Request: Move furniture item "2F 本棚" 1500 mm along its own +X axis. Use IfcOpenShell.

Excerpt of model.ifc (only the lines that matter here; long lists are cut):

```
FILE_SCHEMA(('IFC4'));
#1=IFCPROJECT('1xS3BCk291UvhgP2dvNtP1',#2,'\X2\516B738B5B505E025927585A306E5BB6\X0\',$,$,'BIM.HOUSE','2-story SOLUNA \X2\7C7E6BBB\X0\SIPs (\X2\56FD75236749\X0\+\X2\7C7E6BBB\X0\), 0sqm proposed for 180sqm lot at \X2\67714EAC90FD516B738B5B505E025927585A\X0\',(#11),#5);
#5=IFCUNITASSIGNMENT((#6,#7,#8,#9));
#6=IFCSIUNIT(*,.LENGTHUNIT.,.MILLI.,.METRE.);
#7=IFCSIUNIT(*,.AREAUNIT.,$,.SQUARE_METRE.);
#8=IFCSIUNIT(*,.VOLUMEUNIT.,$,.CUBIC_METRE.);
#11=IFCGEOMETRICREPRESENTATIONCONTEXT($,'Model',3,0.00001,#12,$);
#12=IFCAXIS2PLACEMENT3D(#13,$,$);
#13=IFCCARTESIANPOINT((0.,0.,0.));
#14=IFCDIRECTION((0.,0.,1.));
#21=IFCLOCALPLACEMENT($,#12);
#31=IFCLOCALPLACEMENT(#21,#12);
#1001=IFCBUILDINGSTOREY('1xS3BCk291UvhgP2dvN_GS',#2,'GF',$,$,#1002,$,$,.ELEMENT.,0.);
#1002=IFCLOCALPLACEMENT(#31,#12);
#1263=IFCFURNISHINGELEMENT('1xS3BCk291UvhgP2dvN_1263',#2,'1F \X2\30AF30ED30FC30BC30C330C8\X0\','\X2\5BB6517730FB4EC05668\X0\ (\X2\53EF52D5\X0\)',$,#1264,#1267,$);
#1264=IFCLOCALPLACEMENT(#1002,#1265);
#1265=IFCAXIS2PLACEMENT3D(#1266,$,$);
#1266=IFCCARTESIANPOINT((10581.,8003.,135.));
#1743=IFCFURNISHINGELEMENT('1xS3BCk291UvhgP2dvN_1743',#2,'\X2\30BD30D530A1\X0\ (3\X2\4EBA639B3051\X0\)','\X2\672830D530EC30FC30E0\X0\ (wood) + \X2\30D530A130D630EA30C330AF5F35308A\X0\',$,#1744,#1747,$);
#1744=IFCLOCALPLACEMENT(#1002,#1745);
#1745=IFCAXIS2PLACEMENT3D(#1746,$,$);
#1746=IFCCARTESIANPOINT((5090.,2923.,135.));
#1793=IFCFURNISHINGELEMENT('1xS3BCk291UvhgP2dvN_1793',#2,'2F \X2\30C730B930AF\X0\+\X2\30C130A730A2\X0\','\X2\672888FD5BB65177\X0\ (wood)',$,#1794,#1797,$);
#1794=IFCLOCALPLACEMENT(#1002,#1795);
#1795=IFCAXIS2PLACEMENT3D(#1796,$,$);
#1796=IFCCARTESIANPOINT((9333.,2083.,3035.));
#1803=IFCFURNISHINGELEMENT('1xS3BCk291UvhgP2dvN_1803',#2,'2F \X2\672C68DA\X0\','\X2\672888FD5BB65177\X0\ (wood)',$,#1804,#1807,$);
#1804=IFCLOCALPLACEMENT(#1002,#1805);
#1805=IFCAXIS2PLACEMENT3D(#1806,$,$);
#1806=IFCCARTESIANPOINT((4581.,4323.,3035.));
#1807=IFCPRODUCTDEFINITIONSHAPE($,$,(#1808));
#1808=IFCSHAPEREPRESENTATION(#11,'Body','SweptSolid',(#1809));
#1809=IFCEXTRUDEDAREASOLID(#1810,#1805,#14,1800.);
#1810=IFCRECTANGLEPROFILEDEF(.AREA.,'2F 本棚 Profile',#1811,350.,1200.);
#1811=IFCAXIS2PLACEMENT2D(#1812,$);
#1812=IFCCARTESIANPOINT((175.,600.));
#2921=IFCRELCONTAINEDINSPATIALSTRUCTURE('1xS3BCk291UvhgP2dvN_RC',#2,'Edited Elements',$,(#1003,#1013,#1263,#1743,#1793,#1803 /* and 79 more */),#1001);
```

```python
import ifcopenshell
import ifcopenshell.api.geometry
import ifcopenshell.util.placement
import ifcopenshell.util.unit

model = ifcopenshell.open("model.ifc")
unit_scale = ifcopenshell.util.unit.calculate_unit_scale(model)

item = model.by_guid("1xS3BCk291UvhgP2dvN_1803")
matrix = ifcopenshell.util.placement.get_local_placement(item.ObjectPlacement)
matrix[:3, 3] += matrix[:3, 0] * 1.5 / unit_scale
ifcopenshell.api.geometry.edit_object_placement(model, product=item, matrix=matrix, is_si=False)

print(ifcopenshell.util.placement.get_local_placement(item.ObjectPlacement).round(3) + 0.0)

model.write("model_edited.ifc")
```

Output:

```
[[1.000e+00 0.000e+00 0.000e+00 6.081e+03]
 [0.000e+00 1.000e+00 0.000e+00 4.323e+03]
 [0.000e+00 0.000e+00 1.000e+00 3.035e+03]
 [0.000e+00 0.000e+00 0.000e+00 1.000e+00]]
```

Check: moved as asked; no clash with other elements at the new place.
